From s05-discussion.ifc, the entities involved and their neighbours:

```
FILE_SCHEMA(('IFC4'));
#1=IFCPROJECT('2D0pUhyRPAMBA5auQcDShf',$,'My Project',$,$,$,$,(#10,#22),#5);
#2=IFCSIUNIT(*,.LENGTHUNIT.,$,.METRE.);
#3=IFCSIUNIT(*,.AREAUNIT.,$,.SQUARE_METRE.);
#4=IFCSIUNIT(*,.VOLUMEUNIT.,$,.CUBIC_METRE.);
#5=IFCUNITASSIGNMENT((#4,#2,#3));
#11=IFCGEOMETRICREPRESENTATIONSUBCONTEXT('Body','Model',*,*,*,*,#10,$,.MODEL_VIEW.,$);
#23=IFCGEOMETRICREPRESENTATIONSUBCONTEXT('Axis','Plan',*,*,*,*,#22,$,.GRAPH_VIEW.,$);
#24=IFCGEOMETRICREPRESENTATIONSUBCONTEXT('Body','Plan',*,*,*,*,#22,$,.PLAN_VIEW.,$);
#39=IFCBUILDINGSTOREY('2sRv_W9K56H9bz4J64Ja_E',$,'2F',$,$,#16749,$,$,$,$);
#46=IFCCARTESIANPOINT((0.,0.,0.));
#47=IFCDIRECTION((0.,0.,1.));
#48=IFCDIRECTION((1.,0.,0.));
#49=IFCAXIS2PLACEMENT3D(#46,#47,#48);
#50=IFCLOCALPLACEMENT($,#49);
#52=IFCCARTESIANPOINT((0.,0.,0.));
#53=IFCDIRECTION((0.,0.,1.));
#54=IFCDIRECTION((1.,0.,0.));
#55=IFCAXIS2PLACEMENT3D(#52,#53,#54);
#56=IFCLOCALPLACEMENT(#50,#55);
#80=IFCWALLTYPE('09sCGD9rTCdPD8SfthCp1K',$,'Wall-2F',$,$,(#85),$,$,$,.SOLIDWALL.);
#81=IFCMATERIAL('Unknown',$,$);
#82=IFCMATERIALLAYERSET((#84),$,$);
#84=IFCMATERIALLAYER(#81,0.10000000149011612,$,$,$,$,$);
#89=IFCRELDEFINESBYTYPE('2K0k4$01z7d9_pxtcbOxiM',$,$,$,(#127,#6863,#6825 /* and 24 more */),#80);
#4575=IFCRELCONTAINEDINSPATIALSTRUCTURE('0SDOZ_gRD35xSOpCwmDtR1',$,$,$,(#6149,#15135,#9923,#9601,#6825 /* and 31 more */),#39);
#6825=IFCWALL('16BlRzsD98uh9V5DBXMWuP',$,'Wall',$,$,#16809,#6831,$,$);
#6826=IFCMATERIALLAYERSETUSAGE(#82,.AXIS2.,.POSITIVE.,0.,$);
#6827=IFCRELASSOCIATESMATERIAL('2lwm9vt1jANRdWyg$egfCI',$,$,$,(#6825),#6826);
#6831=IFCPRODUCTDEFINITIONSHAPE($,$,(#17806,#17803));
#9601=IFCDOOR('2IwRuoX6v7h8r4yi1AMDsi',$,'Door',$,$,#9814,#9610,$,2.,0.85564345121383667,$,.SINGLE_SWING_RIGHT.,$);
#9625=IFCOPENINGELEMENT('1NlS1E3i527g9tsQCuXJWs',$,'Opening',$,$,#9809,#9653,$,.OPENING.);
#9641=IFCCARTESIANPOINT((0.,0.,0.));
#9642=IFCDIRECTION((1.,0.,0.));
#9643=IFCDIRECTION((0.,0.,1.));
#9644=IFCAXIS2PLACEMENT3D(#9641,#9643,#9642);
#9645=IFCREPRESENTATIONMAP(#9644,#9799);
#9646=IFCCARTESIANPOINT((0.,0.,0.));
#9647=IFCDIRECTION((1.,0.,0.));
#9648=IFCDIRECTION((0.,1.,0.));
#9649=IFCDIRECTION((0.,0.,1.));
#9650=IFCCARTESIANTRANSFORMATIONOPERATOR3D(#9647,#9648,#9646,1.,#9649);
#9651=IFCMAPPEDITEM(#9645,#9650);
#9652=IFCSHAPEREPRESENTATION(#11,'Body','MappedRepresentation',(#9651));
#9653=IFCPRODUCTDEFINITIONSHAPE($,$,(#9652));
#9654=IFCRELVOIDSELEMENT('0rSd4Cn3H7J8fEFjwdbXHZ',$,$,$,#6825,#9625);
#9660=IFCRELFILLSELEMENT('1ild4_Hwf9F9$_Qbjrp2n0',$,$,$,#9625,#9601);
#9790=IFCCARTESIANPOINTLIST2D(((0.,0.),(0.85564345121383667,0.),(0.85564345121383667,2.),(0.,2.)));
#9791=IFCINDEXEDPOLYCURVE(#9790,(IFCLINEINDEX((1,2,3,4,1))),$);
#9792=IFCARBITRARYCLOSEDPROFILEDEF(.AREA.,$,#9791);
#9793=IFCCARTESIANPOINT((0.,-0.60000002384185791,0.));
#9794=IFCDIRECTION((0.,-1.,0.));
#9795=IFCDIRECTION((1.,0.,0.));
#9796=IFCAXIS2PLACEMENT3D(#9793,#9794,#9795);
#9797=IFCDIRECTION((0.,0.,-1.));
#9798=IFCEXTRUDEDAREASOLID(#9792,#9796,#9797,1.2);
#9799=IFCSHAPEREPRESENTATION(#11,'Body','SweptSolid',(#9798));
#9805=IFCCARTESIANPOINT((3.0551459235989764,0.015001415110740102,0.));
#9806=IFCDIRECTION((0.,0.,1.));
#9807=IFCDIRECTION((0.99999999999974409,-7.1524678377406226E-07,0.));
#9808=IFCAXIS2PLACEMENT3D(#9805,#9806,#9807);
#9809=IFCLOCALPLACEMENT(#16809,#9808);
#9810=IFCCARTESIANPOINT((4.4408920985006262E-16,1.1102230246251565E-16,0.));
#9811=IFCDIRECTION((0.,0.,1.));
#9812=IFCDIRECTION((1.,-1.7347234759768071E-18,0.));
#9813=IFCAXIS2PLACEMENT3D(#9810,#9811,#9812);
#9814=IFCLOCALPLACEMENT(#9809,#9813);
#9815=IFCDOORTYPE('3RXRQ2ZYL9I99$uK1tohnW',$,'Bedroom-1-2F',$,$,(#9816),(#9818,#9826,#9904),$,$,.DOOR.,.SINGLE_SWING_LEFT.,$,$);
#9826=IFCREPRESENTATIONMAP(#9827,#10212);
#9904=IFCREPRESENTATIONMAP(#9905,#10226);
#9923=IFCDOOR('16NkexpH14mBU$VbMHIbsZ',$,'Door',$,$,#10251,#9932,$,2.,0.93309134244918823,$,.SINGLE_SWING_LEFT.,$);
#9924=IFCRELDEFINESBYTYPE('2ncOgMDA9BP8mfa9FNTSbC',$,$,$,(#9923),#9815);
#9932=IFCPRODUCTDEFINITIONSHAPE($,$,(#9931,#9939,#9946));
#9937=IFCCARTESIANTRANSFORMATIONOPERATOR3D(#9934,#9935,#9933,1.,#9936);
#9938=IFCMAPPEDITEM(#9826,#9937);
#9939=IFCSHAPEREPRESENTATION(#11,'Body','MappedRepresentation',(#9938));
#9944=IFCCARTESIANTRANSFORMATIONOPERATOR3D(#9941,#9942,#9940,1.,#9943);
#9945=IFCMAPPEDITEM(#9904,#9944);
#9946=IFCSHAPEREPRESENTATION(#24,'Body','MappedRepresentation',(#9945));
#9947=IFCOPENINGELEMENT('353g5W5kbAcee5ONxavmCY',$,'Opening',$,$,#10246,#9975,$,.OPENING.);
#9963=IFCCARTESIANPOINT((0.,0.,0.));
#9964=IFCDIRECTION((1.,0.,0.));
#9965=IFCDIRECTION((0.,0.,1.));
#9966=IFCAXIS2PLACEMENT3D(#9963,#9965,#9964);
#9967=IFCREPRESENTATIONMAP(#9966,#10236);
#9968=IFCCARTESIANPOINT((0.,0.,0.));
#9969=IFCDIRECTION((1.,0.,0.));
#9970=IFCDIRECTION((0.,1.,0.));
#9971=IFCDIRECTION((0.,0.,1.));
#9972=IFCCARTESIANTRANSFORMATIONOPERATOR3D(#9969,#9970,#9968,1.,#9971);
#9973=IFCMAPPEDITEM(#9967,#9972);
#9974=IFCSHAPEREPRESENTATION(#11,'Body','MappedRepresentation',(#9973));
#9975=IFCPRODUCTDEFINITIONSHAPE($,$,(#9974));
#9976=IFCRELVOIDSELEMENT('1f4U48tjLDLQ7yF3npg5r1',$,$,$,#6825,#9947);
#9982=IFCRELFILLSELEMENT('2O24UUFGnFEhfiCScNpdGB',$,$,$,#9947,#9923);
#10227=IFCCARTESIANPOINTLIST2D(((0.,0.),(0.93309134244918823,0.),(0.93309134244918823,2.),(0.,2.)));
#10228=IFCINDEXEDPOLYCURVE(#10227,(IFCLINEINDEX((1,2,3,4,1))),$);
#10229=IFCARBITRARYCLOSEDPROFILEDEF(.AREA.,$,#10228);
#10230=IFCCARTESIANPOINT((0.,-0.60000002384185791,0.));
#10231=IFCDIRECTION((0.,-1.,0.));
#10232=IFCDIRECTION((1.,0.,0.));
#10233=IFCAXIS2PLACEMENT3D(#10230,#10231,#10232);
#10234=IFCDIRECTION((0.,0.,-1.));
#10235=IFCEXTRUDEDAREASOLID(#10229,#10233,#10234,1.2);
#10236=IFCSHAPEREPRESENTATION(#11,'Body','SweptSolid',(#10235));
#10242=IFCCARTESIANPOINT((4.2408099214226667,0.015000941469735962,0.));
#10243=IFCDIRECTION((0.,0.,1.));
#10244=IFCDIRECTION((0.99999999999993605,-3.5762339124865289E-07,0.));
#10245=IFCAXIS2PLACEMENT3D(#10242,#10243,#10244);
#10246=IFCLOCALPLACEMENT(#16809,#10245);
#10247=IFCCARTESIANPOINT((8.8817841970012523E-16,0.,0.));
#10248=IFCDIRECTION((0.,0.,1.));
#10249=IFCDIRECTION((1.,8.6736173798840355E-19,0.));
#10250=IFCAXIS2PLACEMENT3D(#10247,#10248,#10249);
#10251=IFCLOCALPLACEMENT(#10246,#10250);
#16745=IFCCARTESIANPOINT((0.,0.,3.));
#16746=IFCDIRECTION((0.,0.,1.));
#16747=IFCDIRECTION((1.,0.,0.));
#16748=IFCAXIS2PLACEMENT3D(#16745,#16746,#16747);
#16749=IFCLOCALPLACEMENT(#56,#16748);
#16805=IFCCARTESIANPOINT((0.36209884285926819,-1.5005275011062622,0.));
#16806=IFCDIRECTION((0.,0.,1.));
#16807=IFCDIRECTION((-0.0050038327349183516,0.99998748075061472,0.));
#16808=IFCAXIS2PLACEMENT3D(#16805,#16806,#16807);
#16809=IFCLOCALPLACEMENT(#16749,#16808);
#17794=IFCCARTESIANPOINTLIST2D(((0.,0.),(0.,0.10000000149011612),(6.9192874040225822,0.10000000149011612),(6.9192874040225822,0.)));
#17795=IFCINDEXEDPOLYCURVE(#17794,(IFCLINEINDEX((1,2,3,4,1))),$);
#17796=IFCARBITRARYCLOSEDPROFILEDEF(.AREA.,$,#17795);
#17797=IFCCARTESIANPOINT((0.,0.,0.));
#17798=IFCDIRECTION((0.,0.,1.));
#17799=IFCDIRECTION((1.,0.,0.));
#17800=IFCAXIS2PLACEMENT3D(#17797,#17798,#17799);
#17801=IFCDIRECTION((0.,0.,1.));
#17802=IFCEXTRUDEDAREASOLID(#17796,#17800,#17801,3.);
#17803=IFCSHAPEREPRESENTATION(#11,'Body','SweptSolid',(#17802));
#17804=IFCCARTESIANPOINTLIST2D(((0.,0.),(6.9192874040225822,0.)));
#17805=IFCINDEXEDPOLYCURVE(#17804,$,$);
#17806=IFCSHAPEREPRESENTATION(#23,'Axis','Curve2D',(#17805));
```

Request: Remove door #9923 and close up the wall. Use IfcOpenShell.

```python
import ifcopenshell
import ifcopenshell.api.feature
import ifcopenshell.api.root
import ifcopenshell.geom
import ifcopenshell.util.shape

model = ifcopenshell.open("s05-discussion.ifc")
settings = ifcopenshell.geom.settings()


def volume(element):
    """Net volume in cubic metres, openings subtracted."""
    shape = ifcopenshell.geom.create_shape(settings, element)
    return ifcopenshell.util.shape.get_volume(shape.geometry)


door = model.by_guid("16NkexpH14mBU$VbMHIbsZ")
opening = door.FillsVoids[0].RelatingOpeningElement
wall = opening.VoidsElements[0].RelatingBuildingElement
before = volume(wall)

ifcopenshell.api.root.remove_product(model, product=door)
ifcopenshell.api.feature.remove_feature(model, feature=opening)

after = volume(wall)

print(f"wall volume {before:.3f} -> {after:.3f} m3")

model.write("s05-discussion_edited.ifc")
```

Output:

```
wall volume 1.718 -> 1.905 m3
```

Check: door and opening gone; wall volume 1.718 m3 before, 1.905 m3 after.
